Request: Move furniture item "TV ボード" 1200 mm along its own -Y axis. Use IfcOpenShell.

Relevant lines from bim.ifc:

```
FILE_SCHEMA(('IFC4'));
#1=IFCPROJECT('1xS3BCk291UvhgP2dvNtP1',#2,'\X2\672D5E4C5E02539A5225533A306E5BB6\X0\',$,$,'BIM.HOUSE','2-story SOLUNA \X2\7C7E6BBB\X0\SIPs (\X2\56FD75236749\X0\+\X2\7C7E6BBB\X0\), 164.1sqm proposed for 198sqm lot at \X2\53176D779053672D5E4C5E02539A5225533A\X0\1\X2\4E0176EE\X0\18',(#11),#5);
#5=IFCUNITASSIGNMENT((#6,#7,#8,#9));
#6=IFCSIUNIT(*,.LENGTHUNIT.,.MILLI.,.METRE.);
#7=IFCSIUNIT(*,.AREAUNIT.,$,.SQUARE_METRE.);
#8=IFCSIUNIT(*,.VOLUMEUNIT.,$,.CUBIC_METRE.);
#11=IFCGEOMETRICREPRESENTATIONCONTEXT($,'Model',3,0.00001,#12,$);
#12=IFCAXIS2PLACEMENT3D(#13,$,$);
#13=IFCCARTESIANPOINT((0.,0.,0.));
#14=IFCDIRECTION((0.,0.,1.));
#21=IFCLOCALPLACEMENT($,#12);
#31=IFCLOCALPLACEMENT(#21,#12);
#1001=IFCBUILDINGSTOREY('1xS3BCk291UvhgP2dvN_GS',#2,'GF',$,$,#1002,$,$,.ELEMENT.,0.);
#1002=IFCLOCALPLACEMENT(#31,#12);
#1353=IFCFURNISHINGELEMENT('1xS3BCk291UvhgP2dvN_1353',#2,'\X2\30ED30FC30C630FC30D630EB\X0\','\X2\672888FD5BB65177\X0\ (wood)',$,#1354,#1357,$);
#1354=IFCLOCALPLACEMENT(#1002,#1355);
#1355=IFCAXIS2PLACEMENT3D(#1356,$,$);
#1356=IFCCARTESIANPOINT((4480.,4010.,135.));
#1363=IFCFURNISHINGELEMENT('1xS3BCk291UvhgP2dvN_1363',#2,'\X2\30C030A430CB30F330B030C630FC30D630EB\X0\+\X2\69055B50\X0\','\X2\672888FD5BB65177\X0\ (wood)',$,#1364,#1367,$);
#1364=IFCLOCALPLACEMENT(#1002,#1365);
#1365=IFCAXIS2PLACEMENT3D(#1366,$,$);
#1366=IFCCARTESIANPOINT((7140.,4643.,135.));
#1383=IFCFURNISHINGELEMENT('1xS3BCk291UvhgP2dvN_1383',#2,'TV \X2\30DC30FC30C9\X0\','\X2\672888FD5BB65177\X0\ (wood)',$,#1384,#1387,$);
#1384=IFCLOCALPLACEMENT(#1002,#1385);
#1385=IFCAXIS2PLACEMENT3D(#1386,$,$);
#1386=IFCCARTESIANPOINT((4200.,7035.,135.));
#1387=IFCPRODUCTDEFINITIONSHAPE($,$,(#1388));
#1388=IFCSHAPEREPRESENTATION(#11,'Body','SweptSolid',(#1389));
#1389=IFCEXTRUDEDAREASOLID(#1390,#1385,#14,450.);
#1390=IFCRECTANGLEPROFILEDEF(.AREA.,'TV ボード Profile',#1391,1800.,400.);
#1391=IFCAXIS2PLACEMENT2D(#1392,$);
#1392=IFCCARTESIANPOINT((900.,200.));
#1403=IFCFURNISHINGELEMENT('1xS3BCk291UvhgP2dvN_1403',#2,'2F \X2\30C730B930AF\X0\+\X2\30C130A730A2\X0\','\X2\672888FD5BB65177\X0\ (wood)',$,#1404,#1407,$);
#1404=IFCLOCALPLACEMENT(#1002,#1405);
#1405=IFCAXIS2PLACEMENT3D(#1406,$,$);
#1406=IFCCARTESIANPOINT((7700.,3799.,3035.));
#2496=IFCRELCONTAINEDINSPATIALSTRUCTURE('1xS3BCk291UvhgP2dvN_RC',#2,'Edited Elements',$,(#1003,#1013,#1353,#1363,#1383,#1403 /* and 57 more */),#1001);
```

```python
import ifcopenshell
import ifcopenshell.api.geometry
import ifcopenshell.util.placement

model = ifcopenshell.open("bim.ifc")

item = model.by_guid("1xS3BCk291UvhgP2dvN_1383")
matrix = ifcopenshell.util.placement.get_local_placement(item.ObjectPlacement)
matrix[:3, 3] -= matrix[:3, 1] * 1200.0
ifcopenshell.api.geometry.edit_object_placement(model, product=item, matrix=matrix, is_si=False)

print(ifcopenshell.util.placement.get_local_placement(item.ObjectPlacement).round(3) + 0.0)

model.write("bim_edited.ifc")
```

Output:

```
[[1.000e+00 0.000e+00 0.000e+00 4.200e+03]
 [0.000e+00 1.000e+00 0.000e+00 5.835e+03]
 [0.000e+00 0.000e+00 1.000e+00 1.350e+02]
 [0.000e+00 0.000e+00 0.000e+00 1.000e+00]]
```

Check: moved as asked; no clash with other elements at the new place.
